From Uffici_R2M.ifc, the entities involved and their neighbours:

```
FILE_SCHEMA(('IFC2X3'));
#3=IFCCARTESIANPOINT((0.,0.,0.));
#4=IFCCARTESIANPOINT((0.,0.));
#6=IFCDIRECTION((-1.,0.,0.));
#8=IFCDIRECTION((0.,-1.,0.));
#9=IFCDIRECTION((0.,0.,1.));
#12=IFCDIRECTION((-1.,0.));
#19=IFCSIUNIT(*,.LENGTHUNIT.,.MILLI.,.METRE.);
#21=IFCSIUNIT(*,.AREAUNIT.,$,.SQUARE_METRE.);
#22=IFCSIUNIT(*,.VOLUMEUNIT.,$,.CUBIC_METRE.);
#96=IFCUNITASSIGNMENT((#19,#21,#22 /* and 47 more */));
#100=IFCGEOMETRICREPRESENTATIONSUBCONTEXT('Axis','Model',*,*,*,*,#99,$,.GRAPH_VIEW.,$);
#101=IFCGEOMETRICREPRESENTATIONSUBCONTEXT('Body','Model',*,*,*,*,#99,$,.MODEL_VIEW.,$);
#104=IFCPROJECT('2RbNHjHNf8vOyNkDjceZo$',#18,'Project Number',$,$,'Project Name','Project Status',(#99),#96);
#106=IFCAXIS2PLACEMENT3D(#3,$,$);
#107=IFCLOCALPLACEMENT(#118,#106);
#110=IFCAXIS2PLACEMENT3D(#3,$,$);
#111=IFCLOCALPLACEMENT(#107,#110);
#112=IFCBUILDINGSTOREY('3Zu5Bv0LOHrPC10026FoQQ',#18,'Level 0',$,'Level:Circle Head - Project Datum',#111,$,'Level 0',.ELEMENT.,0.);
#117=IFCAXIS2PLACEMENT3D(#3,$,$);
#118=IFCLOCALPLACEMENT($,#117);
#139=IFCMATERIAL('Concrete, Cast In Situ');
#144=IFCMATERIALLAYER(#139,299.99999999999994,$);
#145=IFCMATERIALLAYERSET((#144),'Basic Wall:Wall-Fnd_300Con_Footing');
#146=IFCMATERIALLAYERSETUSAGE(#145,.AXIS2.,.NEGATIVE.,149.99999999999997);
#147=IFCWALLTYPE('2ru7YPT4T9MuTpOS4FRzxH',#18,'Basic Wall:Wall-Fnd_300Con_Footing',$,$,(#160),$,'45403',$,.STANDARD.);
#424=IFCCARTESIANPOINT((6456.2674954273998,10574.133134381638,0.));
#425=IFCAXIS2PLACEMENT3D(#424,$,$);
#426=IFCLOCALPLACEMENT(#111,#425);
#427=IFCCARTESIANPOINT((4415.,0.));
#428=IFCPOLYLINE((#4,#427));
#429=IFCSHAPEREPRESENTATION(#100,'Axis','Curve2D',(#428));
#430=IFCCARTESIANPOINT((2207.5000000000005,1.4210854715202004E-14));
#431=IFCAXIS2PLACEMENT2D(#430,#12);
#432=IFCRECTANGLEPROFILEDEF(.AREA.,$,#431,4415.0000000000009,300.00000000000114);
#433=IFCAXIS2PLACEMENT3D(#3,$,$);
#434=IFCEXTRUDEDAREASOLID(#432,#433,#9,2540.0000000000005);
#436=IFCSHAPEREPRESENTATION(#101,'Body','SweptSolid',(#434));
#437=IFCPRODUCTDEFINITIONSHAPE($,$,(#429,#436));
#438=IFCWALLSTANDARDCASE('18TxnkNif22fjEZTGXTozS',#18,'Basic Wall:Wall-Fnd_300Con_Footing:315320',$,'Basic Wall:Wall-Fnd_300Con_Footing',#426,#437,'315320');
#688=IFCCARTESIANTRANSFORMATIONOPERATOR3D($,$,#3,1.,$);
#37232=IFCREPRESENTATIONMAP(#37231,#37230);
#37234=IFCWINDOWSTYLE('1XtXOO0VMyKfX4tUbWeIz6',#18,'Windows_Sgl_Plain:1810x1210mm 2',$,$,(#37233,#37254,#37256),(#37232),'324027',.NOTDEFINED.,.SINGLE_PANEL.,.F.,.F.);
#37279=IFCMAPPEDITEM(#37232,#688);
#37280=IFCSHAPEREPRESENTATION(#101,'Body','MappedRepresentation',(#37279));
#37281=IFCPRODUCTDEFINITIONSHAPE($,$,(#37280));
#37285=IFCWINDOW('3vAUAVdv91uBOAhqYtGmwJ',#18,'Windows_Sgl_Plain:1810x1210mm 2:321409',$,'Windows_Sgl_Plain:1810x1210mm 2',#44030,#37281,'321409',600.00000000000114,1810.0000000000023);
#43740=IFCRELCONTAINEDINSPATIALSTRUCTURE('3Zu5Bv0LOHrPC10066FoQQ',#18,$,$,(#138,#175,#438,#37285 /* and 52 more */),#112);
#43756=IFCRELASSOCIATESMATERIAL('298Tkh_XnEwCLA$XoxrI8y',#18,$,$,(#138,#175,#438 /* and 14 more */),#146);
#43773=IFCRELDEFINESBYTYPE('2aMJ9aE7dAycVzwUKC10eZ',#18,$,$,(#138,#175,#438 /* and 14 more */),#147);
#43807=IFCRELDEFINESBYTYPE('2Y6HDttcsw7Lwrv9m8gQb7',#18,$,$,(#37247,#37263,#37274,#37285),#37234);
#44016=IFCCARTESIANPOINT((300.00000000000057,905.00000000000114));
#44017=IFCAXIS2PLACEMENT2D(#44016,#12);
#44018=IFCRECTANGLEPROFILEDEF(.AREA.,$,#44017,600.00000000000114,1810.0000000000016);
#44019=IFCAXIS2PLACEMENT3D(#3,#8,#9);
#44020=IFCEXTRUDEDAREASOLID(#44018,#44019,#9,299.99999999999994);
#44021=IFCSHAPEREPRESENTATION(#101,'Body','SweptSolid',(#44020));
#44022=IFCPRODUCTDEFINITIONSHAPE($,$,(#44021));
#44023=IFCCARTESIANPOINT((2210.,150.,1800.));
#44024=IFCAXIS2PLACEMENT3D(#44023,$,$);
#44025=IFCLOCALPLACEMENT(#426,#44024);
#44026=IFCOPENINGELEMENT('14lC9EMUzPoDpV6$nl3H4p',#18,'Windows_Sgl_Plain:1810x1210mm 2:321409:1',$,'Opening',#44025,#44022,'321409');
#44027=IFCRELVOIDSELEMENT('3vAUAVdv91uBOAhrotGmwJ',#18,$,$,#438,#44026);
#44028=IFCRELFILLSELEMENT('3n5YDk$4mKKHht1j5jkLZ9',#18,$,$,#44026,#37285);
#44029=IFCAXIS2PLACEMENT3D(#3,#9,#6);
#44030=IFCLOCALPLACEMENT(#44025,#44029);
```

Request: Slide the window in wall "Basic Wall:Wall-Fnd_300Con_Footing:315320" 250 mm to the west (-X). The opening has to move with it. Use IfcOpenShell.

```python
import ifcopenshell
import ifcopenshell.api.geometry
import ifcopenshell.util.placement
import ifcopenshell.util.unit

model = ifcopenshell.open("Uffici_R2M.ifc")
unit_scale = ifcopenshell.util.unit.calculate_unit_scale(model)

window = model.by_guid("3vAUAVdv91uBOAhqYtGmwJ")
opening = window.FillsVoids[0].RelatingOpeningElement
wall = opening.VoidsElements[0].RelatingBuildingElement

wall_matrix = ifcopenshell.util.placement.get_local_placement(wall.ObjectPlacement)
shift = wall_matrix[:3, 0] * -0.25 / unit_scale
before = ifcopenshell.util.placement.get_local_placement(window.ObjectPlacement)[:3, 3].copy()

# The window is placed relative to its opening, so it follows when the opening moves.
matrix = ifcopenshell.util.placement.get_local_placement(opening.ObjectPlacement)
matrix[:3, 3] += shift
ifcopenshell.api.geometry.edit_object_placement(
    model, product=opening, matrix=matrix, is_si=False, should_transform_children=True
)

after = ifcopenshell.util.placement.get_local_placement(window.ObjectPlacement)[:3, 3]
print("window moved by", (after - before).round(3) + 0.0)

model.write("Uffici_R2M-out.ifc")
```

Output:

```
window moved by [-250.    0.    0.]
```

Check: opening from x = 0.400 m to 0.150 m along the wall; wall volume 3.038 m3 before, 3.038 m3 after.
